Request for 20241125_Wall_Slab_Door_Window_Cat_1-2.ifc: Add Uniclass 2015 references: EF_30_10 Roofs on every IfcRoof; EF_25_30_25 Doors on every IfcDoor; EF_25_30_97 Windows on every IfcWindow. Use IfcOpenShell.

First a look at what the model holds.

```python
import ifcopenshell

model = ifcopenshell.open("20241125_Wall_Slab_Door_Window_Cat_1-2.ifc")
print(model.schema)
print("classifications:", [c.Name for c in model.by_type("IfcClassification")])
for ifc_class in ("IfcDoor", "IfcRoof", "IfcStair", "IfcWall", "IfcWindow"):
    print(ifc_class, len(model.by_type(ifc_class)))
```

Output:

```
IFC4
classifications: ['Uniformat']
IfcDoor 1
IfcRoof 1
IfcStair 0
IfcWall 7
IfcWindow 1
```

```python
import ifcopenshell
import ifcopenshell.api.classification

model = ifcopenshell.open("20241125_Wall_Slab_Door_Window_Cat_1-2.ifc")

system = ifcopenshell.api.classification.add_classification(model, classification="Uniclass 2015")

codes = {
    "IfcRoof": ("EF_30_10", "Roofs"),
    "IfcDoor": ("EF_25_30_25", "Doors"),
    "IfcWindow": ("EF_25_30_97", "Windows"),
}
for ifc_class, (code, name) in codes.items():
    products = model.by_type(ifc_class)
    ifcopenshell.api.classification.add_reference(
        model, products=products, classification=system, identification=code, name=name
    )
    print(code, len(products))

model.write("20241125_Wall_Slab_Door_Window_Cat_1-2_rev.ifc")
```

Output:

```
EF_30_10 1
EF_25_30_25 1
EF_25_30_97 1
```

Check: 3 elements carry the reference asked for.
